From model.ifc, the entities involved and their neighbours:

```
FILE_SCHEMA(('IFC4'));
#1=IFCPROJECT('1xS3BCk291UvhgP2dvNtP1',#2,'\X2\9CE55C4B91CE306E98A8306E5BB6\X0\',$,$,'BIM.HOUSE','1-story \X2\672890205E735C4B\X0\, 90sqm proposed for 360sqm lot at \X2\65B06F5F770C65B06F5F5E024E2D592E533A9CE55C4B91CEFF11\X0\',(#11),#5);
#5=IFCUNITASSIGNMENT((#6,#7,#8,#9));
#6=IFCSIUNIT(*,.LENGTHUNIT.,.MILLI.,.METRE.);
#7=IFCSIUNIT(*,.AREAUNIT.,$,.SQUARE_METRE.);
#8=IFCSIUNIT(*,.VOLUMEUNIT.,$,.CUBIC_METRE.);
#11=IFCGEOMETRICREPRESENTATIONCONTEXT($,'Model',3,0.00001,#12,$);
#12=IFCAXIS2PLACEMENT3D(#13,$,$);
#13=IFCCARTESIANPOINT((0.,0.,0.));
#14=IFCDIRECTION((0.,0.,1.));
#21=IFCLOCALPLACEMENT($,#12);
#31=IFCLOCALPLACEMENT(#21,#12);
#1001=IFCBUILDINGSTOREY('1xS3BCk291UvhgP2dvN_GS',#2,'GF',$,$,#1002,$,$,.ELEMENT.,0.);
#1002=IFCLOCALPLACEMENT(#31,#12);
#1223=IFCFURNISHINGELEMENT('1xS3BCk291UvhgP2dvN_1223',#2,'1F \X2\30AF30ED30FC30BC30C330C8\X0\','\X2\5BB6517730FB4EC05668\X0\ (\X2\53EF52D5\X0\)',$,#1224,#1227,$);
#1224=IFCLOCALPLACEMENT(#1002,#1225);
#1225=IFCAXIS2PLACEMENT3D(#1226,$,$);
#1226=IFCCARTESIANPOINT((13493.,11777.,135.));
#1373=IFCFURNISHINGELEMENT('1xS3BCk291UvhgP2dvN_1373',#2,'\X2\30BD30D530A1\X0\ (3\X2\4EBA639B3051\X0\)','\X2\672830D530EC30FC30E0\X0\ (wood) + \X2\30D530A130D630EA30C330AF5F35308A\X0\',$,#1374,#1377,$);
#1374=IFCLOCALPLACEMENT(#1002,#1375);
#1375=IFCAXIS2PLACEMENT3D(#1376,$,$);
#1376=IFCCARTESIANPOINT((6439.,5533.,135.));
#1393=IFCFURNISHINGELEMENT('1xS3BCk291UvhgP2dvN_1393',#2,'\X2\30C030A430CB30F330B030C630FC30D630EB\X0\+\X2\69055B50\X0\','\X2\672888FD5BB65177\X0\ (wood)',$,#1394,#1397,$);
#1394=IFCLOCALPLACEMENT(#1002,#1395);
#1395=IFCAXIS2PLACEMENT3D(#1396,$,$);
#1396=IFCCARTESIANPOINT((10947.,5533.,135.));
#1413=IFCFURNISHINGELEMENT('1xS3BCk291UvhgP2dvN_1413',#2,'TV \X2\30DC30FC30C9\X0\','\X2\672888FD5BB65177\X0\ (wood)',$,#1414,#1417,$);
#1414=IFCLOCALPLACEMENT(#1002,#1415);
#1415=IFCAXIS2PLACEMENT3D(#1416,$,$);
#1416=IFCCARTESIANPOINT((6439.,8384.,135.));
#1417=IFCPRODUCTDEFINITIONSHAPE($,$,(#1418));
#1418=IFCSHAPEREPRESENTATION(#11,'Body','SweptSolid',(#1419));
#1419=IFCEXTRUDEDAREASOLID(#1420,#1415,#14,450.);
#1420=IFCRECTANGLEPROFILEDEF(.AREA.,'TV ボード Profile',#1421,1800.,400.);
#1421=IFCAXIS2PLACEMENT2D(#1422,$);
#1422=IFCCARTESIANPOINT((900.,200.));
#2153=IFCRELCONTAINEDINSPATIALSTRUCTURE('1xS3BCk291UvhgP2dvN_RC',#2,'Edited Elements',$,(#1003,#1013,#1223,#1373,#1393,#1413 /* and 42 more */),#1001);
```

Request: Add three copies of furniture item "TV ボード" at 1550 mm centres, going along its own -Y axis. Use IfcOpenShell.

```python
import ifcopenshell
import ifcopenshell.api.geometry
import ifcopenshell.api.root
import ifcopenshell.util.element
import ifcopenshell.util.placement
import ifcopenshell.util.unit

model = ifcopenshell.open("model.ifc")
unit_scale = ifcopenshell.util.unit.calculate_unit_scale(model)


def reuse_history(source, copy):
    """copy_class also copies each property set's owner history, people and application; keep the originals."""
    for rel in copy.IsDefinedBy:
        if rel.is_a("IfcRelDefinesByProperties") and (history := rel.RelatingPropertyDefinition.OwnerHistory):
            rel.RelatingPropertyDefinition.OwnerHistory = source.OwnerHistory
            ifcopenshell.util.element.remove_deep2(model, history)


source = model.by_guid("1xS3BCk291UvhgP2dvN_1413")
base = ifcopenshell.util.placement.get_local_placement(source.ObjectPlacement)
step = -base[:3, 1] * 1.55 / unit_scale

for i in range(1, 4):
    copy = ifcopenshell.api.root.copy_class(model, product=source)
    copy.Representation = ifcopenshell.util.element.copy_deep(
        model, source.Representation, exclude=["IfcGeometricRepresentationContext", "IfcRepresentationMap"]
    )
    reuse_history(source, copy)
    matrix = base.copy()
    matrix[:3, 3] += i * step
    print("added at", matrix[:3, 3].round(3) + 0.0)
    ifcopenshell.api.geometry.edit_object_placement(model, product=copy, matrix=matrix, is_si=False)

model.write("model_edited.ifc")
```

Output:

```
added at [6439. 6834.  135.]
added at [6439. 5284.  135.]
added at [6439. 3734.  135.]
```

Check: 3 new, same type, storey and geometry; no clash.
